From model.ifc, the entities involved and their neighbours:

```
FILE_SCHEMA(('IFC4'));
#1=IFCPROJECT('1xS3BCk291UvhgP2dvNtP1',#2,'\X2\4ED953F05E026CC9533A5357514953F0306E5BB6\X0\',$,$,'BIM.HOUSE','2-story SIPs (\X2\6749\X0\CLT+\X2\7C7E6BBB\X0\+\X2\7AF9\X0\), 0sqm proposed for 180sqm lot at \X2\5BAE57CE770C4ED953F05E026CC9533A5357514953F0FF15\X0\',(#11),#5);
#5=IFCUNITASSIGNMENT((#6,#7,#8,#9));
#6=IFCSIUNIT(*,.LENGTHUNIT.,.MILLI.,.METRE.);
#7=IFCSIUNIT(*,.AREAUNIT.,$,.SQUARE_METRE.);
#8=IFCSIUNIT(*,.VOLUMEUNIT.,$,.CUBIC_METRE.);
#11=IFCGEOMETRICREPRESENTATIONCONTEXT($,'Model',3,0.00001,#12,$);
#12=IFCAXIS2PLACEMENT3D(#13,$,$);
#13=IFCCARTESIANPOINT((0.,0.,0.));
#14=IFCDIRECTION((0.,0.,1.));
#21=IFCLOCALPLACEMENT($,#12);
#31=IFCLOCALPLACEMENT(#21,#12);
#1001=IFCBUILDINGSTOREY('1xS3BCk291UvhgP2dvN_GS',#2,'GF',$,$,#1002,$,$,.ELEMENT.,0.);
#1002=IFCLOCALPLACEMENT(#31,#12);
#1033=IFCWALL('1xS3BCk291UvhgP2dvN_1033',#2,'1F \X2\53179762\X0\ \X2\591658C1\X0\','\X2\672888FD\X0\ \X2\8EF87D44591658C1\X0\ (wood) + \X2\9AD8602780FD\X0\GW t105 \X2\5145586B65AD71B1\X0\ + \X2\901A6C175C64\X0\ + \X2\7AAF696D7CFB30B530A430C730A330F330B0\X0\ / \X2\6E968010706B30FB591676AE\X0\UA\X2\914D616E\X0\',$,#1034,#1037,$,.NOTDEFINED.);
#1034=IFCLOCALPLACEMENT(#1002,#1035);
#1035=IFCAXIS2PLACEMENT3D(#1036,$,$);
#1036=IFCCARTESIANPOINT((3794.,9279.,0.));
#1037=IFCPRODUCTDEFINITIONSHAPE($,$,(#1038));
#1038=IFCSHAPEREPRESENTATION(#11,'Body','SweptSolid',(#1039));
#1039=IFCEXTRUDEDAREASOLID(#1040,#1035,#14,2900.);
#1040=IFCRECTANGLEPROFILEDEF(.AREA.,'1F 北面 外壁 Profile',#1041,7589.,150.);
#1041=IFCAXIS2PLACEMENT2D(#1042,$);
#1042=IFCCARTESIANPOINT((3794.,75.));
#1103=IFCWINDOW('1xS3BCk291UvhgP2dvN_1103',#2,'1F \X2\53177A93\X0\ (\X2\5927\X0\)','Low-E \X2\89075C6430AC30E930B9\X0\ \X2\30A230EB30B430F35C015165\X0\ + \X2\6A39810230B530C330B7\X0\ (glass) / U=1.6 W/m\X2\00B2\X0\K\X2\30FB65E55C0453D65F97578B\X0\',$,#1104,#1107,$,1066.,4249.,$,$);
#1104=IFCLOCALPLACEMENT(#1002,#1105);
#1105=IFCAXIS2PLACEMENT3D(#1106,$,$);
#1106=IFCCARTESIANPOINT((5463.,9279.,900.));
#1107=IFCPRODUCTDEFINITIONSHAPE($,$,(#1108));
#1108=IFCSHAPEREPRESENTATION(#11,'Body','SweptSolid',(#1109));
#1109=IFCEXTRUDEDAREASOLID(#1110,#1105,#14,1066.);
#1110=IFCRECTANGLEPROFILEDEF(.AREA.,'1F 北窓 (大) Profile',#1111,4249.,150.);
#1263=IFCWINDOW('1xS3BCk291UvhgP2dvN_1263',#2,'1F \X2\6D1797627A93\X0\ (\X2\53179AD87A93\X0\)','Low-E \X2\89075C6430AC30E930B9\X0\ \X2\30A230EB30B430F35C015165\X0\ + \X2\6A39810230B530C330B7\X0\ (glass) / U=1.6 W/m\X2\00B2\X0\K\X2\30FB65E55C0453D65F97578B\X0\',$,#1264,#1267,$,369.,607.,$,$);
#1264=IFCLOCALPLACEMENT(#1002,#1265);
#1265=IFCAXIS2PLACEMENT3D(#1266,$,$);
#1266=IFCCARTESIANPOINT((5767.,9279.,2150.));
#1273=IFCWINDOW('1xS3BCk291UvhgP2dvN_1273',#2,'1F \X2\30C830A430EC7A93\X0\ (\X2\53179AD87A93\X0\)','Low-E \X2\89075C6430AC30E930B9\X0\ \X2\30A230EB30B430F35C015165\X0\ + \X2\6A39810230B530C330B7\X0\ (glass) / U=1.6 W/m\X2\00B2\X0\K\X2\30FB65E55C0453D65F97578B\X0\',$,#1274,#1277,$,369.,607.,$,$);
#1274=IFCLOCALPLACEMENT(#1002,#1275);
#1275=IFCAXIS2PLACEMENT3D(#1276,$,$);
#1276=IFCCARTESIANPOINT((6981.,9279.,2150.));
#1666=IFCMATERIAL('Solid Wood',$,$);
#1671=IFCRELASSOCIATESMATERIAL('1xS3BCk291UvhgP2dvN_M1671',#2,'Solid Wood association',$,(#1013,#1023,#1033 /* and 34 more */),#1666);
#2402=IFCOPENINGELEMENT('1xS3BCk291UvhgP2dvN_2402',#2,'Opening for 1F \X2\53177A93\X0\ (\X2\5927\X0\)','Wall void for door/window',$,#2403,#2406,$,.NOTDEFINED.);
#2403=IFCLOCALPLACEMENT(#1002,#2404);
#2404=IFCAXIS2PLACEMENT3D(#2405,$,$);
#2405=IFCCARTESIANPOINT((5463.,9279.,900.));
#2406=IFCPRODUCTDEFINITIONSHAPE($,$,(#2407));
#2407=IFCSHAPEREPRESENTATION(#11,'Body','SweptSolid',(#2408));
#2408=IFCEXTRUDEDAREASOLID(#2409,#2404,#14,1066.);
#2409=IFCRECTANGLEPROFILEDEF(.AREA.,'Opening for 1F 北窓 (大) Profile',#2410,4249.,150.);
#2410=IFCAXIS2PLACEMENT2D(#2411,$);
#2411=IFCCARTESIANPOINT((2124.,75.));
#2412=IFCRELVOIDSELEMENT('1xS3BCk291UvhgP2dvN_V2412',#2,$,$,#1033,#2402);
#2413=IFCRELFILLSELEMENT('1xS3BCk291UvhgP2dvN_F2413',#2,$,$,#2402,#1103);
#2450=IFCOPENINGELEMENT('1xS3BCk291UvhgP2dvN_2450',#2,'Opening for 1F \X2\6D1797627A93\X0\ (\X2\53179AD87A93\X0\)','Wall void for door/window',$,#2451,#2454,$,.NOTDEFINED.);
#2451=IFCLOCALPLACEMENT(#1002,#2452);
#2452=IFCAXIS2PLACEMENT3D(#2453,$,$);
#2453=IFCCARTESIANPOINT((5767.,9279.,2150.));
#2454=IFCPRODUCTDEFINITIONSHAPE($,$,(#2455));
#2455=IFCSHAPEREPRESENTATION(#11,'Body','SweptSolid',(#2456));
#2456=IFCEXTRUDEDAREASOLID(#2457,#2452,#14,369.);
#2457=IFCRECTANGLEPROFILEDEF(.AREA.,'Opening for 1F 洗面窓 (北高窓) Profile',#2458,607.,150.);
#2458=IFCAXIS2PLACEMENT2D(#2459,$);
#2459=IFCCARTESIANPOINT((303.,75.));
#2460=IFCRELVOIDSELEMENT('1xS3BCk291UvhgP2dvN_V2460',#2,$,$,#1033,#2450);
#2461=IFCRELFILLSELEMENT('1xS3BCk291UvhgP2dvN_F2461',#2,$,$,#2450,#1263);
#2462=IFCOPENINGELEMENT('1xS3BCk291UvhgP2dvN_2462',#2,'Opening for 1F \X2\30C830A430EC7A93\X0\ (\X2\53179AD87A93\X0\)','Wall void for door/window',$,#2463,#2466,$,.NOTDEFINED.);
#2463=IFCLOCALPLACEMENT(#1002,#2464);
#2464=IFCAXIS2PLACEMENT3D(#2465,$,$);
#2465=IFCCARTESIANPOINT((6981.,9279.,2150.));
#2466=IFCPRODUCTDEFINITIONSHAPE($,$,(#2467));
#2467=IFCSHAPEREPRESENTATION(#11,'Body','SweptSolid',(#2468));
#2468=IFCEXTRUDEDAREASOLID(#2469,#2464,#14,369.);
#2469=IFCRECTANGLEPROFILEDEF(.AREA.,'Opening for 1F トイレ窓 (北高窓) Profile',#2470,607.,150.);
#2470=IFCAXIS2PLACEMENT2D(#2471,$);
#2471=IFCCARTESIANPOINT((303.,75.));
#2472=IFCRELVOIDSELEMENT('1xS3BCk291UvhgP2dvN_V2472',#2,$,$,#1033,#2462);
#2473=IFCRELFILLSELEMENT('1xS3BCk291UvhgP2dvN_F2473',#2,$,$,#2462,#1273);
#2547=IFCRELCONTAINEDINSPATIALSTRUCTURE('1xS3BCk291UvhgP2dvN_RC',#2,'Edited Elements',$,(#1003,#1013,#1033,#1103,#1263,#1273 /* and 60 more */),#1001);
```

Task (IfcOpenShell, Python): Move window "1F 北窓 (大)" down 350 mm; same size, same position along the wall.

```python
import numpy as np
import ifcopenshell
import ifcopenshell.api.geometry
import ifcopenshell.util.placement
import ifcopenshell.util.unit

model = ifcopenshell.open("model.ifc")
unit_scale = ifcopenshell.util.unit.calculate_unit_scale(model)

window = model.by_id(1103)
opening = window.FillsVoids[0].RelatingOpeningElement
dz = -0.35 / unit_scale

shift = np.array([0.0, 0.0, dz])
# The window is not placed relative to its opening, so move both.
for product in (opening, window):
    matrix = ifcopenshell.util.placement.get_local_placement(product.ObjectPlacement)
    matrix[:3, 3] += shift
    ifcopenshell.api.geometry.edit_object_placement(model, product=product, matrix=matrix, is_si=False)

print(f"moved by {dz * unit_scale:+.3f} m")

model.write("model_edited.ifc")
```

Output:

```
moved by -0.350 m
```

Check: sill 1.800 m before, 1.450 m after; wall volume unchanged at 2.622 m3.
